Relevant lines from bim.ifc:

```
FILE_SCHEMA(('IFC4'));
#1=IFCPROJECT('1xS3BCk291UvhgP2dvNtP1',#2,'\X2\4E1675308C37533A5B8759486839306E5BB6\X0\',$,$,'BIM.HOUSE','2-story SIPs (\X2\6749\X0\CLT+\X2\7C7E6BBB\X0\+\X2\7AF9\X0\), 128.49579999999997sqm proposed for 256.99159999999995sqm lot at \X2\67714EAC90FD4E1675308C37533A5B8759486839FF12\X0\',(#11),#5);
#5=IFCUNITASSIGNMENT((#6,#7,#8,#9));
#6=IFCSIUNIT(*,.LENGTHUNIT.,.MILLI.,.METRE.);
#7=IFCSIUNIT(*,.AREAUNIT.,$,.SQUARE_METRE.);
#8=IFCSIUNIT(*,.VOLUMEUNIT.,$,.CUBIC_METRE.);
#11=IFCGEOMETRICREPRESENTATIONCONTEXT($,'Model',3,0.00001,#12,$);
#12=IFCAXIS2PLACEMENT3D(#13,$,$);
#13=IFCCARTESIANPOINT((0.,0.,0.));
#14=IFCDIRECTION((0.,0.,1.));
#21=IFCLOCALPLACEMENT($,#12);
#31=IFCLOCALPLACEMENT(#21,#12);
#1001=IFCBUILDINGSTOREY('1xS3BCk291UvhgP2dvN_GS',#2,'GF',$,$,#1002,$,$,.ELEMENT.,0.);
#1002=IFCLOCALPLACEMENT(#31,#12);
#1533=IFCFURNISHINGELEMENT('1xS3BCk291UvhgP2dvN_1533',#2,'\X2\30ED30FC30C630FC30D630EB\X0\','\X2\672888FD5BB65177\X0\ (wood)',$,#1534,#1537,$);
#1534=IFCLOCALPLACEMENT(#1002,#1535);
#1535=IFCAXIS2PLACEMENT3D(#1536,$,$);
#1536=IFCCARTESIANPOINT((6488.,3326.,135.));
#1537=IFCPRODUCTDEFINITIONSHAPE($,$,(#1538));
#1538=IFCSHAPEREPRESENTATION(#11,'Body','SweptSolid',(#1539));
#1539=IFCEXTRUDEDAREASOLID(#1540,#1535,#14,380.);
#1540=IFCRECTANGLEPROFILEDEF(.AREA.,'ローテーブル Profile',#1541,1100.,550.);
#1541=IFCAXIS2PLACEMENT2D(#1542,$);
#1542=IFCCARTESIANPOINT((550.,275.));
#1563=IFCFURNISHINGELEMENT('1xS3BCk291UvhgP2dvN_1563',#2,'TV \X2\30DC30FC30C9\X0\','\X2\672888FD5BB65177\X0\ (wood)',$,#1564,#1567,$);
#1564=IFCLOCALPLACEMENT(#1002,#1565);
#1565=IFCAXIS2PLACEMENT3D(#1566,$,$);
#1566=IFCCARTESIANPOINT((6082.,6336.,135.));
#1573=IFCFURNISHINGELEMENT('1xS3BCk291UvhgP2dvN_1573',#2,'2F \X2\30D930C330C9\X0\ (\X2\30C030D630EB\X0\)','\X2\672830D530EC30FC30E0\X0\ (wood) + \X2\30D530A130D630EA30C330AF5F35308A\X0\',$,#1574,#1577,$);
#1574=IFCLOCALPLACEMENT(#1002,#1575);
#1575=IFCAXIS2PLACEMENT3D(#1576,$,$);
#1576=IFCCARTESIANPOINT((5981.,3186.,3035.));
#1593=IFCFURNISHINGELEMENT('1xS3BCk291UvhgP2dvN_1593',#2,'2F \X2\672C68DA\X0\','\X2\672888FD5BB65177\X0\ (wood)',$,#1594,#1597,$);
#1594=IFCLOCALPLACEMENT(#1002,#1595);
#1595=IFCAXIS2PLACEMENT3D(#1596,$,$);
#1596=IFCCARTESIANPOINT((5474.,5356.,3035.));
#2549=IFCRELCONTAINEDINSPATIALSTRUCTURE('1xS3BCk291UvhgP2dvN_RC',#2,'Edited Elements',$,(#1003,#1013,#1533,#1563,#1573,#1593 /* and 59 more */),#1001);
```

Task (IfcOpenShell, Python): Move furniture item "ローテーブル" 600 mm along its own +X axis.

```python
import ifcopenshell
import ifcopenshell.api.geometry
import ifcopenshell.util.placement
import ifcopenshell.util.unit

model = ifcopenshell.open("bim.ifc")
unit_scale = ifcopenshell.util.unit.calculate_unit_scale(model)

item = model.by_guid("1xS3BCk291UvhgP2dvN_1533")
matrix = ifcopenshell.util.placement.get_local_placement(item.ObjectPlacement)
matrix[:3, 3] += matrix[:3, 0] * 0.6 / unit_scale
ifcopenshell.api.geometry.edit_object_placement(model, product=item, matrix=matrix, is_si=False)

print(ifcopenshell.util.placement.get_local_placement(item.ObjectPlacement).round(3) + 0.0)

model.write("bim_v2.ifc")
```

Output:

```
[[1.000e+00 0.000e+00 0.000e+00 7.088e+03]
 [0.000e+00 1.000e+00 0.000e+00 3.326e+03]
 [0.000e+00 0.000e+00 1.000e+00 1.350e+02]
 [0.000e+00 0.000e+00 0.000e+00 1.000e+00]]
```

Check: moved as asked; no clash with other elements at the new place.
